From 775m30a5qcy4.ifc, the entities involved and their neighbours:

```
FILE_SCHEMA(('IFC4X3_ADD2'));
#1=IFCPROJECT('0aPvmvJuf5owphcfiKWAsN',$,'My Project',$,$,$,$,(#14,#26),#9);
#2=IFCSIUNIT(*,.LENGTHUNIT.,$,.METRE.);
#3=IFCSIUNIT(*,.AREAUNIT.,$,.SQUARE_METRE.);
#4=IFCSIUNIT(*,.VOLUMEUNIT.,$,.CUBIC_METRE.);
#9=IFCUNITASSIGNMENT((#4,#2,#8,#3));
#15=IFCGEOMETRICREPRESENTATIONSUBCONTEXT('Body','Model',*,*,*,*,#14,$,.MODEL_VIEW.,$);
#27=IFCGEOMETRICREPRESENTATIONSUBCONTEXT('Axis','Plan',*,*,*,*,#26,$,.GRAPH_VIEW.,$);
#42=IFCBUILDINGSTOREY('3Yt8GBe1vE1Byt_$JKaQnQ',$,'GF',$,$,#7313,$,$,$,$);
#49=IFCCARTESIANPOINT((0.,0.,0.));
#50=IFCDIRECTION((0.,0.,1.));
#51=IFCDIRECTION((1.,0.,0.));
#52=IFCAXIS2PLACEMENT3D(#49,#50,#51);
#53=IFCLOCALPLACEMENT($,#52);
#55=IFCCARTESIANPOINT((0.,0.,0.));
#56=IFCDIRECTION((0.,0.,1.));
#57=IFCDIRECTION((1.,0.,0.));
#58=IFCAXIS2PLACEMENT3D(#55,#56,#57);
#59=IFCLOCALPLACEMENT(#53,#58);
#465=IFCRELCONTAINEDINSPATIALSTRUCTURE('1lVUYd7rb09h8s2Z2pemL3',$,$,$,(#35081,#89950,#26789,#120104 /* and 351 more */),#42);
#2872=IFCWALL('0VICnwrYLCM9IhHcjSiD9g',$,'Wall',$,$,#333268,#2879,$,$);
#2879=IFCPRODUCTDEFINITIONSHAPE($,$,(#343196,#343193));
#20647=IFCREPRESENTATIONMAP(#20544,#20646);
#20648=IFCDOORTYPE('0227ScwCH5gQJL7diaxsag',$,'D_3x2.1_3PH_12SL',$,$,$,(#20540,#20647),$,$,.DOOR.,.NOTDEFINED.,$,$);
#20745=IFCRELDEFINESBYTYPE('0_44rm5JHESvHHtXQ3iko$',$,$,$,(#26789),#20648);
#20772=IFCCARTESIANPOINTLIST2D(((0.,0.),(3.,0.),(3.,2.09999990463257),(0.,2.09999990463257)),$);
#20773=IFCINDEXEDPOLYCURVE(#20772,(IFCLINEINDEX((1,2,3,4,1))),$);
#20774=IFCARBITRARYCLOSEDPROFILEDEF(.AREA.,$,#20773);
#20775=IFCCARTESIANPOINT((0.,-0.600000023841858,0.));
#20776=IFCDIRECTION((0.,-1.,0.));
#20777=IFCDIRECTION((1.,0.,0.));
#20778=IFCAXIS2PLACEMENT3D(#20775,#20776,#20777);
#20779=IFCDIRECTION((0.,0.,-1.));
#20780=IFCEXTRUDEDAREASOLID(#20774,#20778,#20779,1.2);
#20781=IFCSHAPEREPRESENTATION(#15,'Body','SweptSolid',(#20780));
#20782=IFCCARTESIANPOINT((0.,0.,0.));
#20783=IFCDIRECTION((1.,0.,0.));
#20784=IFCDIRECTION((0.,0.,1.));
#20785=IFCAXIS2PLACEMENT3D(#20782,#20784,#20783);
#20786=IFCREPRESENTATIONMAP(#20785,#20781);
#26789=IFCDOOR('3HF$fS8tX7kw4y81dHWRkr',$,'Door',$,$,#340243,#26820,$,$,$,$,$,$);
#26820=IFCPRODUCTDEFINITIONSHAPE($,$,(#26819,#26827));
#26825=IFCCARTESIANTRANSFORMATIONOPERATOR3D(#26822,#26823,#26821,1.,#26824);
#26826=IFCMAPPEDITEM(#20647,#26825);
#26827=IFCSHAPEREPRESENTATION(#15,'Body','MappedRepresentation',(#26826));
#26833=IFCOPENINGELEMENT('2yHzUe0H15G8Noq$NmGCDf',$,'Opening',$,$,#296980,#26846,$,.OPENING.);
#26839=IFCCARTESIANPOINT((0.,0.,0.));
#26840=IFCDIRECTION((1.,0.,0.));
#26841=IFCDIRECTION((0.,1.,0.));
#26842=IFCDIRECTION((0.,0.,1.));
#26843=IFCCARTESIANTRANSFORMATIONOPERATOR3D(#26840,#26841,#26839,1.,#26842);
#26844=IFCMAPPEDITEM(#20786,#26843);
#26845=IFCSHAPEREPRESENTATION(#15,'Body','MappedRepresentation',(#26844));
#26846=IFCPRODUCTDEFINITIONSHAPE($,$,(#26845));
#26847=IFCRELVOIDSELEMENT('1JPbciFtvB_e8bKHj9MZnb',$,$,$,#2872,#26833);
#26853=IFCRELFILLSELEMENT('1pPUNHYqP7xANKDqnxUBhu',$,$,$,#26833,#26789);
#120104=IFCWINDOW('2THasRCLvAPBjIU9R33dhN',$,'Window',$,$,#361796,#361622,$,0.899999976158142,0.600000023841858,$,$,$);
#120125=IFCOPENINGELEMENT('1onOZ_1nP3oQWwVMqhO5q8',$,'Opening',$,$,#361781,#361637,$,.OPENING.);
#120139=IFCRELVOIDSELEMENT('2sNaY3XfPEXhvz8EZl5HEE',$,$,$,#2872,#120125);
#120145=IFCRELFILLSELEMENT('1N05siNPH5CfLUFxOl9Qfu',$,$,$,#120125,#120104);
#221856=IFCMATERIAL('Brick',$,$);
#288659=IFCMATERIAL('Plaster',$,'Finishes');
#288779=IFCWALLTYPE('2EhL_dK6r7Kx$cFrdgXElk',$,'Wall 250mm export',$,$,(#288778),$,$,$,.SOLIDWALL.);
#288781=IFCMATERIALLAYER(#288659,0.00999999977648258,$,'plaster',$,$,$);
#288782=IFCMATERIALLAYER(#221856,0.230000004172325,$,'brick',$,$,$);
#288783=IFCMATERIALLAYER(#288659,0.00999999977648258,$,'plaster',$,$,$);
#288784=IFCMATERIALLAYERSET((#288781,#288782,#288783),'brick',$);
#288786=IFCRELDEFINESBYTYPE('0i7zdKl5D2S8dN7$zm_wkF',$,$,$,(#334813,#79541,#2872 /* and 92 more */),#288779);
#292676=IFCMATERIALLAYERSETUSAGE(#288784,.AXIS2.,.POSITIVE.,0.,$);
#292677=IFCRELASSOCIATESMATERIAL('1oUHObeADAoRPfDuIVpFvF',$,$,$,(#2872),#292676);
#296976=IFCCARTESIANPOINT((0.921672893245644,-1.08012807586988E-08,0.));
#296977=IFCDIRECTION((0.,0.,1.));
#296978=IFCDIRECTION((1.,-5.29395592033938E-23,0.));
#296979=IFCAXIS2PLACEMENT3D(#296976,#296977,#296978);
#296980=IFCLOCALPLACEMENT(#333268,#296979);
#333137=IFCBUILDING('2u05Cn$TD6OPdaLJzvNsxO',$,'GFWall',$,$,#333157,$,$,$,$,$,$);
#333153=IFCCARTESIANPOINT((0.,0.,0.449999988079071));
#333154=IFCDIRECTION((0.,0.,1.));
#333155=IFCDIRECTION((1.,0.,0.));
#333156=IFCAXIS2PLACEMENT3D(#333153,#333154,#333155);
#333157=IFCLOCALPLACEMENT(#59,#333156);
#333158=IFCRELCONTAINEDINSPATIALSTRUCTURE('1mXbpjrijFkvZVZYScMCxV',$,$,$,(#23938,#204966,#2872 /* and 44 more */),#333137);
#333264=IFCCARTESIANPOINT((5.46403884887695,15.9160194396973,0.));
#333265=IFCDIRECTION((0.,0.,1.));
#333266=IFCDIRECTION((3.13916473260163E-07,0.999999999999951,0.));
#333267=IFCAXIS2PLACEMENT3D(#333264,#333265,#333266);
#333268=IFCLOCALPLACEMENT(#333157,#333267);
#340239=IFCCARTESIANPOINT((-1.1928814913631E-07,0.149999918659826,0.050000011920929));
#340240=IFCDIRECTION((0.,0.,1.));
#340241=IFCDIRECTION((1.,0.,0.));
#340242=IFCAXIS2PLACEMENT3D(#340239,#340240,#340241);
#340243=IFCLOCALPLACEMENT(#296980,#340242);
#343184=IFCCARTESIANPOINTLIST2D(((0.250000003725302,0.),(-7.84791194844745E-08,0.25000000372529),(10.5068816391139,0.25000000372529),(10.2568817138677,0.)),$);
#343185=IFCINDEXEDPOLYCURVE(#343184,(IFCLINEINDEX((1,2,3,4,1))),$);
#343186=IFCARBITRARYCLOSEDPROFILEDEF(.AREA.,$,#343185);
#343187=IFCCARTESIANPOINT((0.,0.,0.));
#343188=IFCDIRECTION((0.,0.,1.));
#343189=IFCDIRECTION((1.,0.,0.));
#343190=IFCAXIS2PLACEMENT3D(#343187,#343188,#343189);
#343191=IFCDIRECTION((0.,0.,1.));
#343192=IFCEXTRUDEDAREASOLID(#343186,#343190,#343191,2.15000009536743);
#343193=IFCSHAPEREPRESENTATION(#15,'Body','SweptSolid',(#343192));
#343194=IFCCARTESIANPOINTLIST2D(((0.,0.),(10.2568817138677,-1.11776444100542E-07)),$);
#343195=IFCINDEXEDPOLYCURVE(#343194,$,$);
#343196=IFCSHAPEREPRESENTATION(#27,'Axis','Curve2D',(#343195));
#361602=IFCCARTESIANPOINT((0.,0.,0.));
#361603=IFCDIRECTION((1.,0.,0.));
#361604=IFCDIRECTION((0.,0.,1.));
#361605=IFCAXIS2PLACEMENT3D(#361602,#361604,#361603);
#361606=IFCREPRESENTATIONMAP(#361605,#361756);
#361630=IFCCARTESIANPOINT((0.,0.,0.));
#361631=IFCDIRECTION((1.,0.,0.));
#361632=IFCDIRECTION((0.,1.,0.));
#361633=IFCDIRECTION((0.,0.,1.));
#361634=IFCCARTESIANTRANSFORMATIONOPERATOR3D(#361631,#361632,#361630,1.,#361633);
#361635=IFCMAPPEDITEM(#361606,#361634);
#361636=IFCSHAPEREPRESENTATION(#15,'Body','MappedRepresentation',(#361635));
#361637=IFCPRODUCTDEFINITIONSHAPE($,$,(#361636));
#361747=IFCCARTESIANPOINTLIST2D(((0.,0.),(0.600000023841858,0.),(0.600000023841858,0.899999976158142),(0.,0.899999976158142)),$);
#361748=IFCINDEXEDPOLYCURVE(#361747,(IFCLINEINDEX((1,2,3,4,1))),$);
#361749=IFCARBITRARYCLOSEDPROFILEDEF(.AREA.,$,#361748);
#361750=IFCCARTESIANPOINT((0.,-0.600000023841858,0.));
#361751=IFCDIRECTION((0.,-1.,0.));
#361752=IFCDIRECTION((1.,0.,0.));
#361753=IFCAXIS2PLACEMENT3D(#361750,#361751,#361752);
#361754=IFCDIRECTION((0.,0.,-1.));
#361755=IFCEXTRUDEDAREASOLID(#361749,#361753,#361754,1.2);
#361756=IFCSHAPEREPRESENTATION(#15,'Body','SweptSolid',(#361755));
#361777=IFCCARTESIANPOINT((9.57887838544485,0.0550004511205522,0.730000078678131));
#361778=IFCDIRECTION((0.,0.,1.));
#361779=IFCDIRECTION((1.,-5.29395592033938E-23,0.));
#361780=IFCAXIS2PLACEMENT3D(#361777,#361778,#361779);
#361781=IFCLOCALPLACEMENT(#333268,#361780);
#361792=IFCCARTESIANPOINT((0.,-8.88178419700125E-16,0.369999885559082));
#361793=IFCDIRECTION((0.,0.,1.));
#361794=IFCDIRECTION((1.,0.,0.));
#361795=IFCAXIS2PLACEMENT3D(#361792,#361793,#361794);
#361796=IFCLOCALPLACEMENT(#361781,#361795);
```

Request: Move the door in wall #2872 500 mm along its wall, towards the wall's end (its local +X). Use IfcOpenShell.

```python
import ifcopenshell
import ifcopenshell.api.geometry
import ifcopenshell.util.placement

model = ifcopenshell.open("775m30a5qcy4.ifc")

door = model.by_id(26789)
opening = door.FillsVoids[0].RelatingOpeningElement
wall = opening.VoidsElements[0].RelatingBuildingElement

wall_matrix = ifcopenshell.util.placement.get_local_placement(wall.ObjectPlacement)
shift = wall_matrix[:3, 0] * 0.5
before = ifcopenshell.util.placement.get_local_placement(door.ObjectPlacement)[:3, 3].copy()

# The door is placed relative to its opening, so it follows when the opening moves.
matrix = ifcopenshell.util.placement.get_local_placement(opening.ObjectPlacement)
matrix[:3, 3] += shift
ifcopenshell.api.geometry.edit_object_placement(
    model, product=opening, matrix=matrix, is_si=False, should_transform_children=True
)

after = ifcopenshell.util.placement.get_local_placement(door.ObjectPlacement)[:3, 3]
print("door moved by", (after - before).round(3) + 0.0)

model.write("775m30a5qcy4_updated.ifc")
```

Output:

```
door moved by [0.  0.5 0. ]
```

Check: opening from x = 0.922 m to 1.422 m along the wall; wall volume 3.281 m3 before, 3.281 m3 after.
